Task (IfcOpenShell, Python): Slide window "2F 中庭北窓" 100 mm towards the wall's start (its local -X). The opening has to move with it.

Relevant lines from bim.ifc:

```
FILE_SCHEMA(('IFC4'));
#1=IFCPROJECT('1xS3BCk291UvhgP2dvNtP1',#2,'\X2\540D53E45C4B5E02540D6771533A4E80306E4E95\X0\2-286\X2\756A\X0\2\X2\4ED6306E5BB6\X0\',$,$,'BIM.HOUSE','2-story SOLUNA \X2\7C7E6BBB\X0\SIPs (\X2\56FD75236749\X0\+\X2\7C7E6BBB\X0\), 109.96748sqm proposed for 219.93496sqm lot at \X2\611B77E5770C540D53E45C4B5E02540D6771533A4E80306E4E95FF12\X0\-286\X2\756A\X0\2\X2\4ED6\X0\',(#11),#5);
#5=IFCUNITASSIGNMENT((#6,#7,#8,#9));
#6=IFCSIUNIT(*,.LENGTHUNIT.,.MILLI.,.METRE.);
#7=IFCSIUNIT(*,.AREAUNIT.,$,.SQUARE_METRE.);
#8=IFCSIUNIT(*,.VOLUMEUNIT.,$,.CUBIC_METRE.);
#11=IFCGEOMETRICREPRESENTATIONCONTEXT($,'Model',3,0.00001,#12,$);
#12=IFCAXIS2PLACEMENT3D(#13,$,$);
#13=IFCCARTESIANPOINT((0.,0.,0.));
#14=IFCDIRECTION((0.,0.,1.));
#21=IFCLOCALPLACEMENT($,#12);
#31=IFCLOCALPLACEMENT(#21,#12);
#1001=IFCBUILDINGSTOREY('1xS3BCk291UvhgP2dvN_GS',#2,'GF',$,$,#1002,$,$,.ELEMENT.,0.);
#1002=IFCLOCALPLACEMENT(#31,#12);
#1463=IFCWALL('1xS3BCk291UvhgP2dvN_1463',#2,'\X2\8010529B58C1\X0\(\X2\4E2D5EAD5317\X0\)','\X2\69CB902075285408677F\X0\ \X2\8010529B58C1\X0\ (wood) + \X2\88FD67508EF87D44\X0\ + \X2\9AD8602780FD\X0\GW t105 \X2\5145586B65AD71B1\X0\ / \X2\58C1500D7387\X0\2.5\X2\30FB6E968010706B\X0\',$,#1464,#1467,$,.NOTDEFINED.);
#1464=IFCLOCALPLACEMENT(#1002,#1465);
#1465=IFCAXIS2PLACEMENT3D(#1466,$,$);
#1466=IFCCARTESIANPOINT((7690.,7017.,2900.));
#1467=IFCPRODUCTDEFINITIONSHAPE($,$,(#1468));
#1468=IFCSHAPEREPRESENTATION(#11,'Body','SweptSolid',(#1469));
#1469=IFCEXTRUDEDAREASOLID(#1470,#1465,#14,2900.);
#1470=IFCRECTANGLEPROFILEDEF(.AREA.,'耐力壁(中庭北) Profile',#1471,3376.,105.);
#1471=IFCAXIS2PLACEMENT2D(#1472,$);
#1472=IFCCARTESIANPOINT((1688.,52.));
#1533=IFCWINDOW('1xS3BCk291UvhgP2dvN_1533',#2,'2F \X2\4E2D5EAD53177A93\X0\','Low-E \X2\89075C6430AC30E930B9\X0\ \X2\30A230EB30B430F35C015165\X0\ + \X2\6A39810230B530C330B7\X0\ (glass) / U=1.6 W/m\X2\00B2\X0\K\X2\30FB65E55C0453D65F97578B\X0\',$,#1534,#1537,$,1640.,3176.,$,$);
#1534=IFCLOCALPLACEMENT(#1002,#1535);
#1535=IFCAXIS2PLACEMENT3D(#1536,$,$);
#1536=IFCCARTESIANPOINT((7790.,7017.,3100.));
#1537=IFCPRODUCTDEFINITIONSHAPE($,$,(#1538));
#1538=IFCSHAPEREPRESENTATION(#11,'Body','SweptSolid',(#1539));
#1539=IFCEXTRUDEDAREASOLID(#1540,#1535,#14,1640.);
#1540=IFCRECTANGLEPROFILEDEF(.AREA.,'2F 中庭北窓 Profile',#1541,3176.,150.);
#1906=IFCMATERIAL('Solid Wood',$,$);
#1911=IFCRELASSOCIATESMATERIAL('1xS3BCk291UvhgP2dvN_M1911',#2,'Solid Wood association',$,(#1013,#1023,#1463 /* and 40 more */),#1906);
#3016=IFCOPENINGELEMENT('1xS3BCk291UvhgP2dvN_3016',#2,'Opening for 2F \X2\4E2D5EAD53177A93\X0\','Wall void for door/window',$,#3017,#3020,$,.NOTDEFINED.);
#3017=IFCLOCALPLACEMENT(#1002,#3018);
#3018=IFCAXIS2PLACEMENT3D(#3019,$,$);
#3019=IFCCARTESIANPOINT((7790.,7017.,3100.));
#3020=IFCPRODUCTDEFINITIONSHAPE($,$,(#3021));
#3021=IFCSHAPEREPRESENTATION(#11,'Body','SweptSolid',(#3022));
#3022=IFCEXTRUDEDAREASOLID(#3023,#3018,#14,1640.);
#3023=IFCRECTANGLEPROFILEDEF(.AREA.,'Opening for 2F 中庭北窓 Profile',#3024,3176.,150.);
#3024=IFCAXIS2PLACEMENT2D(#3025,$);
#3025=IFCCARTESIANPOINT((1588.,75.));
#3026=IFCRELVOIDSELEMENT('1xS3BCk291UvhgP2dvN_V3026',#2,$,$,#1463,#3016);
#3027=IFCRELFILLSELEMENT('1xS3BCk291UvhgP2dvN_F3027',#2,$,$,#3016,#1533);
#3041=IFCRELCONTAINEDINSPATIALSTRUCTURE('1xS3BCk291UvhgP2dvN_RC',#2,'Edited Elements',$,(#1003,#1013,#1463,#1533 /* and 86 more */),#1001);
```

```python
import ifcopenshell
import ifcopenshell.api.geometry
import ifcopenshell.util.placement

model = ifcopenshell.open("bim.ifc")

window = model.by_guid("1xS3BCk291UvhgP2dvN_1533")
opening = window.FillsVoids[0].RelatingOpeningElement
wall = opening.VoidsElements[0].RelatingBuildingElement

wall_matrix = ifcopenshell.util.placement.get_local_placement(wall.ObjectPlacement)
shift = wall_matrix[:3, 0] * -100.0
before = ifcopenshell.util.placement.get_local_placement(window.ObjectPlacement)[:3, 3].copy()

# The window is not placed relative to its opening, so move both.
for product in (opening, window):
    matrix = ifcopenshell.util.placement.get_local_placement(product.ObjectPlacement)
    matrix[:3, 3] += shift
    ifcopenshell.api.geometry.edit_object_placement(model, product=product, matrix=matrix, is_si=False)

after = ifcopenshell.util.placement.get_local_placement(window.ObjectPlacement)[:3, 3]
print("window moved by", (after - before).round(3) + 0.0)

model.write("bim-out.ifc")
```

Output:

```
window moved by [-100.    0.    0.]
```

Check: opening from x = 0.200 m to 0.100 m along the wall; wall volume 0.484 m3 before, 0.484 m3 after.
